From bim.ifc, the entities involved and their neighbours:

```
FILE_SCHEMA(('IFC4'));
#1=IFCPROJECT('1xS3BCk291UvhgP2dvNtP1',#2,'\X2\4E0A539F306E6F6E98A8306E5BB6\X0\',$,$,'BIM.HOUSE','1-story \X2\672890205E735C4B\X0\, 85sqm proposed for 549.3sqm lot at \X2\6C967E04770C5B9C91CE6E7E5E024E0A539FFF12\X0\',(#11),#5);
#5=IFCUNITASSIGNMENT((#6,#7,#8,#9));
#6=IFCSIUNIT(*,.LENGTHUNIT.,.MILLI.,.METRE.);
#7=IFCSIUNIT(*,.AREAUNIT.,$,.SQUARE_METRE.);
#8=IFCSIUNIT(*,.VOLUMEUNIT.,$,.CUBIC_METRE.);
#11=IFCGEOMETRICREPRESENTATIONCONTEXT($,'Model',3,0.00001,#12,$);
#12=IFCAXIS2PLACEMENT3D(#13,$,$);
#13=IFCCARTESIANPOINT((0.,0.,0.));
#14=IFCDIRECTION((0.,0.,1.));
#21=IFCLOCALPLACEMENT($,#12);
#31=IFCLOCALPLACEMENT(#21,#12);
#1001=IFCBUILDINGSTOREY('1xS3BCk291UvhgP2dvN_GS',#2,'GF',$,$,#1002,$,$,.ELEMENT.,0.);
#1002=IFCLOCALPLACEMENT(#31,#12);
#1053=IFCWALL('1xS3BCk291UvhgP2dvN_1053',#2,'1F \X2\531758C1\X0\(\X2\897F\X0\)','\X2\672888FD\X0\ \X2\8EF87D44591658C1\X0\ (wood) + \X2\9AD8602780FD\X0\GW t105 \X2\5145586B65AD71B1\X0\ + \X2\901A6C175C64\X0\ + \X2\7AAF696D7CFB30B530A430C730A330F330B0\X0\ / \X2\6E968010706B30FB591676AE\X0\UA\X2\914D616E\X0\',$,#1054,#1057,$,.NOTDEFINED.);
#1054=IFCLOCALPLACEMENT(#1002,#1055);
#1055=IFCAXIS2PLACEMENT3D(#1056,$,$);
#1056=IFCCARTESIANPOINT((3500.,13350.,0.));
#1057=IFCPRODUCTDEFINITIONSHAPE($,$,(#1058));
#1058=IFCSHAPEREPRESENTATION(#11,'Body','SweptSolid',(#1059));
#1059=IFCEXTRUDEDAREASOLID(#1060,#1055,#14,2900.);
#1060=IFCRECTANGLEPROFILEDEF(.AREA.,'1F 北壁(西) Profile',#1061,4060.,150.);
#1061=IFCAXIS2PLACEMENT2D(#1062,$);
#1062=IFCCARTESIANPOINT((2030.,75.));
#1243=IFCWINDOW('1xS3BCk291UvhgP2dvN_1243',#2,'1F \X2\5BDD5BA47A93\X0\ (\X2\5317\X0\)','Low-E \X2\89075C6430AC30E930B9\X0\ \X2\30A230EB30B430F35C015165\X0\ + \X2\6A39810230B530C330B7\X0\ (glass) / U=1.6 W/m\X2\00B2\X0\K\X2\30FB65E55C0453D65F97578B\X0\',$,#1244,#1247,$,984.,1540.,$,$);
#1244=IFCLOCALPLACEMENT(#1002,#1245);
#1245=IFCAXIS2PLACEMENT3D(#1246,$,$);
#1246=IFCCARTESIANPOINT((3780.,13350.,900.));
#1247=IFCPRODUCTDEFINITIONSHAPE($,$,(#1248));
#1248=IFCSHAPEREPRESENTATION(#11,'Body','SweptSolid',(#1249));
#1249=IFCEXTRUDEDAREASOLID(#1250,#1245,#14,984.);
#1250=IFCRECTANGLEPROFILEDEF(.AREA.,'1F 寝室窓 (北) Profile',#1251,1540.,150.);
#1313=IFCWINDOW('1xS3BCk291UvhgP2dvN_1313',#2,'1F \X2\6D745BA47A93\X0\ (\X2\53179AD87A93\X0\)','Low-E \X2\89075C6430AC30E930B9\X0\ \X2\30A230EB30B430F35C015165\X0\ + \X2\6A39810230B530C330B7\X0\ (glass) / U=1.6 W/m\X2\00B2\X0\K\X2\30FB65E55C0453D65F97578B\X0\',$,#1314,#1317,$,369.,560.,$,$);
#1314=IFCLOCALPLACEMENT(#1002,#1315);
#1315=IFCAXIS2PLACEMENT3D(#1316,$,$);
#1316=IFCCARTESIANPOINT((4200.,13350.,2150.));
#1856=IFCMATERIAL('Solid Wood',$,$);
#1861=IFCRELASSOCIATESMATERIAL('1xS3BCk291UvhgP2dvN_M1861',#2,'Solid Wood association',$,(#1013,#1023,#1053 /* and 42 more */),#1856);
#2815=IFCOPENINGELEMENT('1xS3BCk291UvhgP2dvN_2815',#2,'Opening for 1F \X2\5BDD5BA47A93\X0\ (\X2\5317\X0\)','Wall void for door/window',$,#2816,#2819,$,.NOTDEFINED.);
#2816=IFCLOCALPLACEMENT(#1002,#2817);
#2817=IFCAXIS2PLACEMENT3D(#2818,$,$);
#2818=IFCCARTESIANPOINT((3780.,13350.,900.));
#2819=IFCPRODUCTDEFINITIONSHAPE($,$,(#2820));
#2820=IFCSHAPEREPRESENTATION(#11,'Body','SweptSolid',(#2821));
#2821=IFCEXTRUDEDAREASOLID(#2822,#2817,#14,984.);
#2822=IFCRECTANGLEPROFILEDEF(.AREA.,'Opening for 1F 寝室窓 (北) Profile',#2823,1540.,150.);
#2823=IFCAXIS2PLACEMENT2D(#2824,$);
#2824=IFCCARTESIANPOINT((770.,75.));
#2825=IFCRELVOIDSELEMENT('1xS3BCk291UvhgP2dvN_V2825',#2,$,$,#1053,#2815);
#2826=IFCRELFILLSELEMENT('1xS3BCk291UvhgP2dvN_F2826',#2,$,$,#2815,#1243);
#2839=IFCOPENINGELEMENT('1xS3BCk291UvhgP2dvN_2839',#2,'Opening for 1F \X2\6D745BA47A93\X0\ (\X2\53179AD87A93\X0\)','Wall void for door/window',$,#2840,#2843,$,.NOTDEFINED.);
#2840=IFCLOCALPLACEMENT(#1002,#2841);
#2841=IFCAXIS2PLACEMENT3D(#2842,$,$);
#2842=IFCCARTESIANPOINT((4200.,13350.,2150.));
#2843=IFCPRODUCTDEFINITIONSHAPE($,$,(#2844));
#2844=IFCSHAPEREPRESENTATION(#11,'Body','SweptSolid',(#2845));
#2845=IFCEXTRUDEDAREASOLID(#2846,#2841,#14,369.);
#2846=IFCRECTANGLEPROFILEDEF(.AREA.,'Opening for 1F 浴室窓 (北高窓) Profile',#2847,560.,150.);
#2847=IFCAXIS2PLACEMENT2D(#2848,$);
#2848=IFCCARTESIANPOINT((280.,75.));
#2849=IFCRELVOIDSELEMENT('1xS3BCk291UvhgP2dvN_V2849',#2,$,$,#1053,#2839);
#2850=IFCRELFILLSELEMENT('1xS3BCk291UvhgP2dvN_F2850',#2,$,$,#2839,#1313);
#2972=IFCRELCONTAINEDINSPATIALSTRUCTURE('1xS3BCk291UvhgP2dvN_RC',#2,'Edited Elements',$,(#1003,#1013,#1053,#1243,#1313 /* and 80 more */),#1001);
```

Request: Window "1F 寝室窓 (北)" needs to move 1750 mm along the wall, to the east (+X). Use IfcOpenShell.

```python
import ifcopenshell
import ifcopenshell.api.geometry
import ifcopenshell.util.placement
import ifcopenshell.util.unit

model = ifcopenshell.open("bim.ifc")
unit_scale = ifcopenshell.util.unit.calculate_unit_scale(model)

window = model.by_guid("1xS3BCk291UvhgP2dvN_1243")
opening = window.FillsVoids[0].RelatingOpeningElement
wall = opening.VoidsElements[0].RelatingBuildingElement

wall_matrix = ifcopenshell.util.placement.get_local_placement(wall.ObjectPlacement)
shift = wall_matrix[:3, 0] * 1.75 / unit_scale
before = ifcopenshell.util.placement.get_local_placement(window.ObjectPlacement)[:3, 3].copy()

# The window is not placed relative to its opening, so move both.
for product in (opening, window):
    matrix = ifcopenshell.util.placement.get_local_placement(product.ObjectPlacement)
    matrix[:3, 3] += shift
    ifcopenshell.api.geometry.edit_object_placement(model, product=product, matrix=matrix, is_si=False)

after = ifcopenshell.util.placement.get_local_placement(window.ObjectPlacement)[:3, 3]
print("window moved by", (after - before).round(3) + 0.0)

model.write("bim_rev.ifc")
```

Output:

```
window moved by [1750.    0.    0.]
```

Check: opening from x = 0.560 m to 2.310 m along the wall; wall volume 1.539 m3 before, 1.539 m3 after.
